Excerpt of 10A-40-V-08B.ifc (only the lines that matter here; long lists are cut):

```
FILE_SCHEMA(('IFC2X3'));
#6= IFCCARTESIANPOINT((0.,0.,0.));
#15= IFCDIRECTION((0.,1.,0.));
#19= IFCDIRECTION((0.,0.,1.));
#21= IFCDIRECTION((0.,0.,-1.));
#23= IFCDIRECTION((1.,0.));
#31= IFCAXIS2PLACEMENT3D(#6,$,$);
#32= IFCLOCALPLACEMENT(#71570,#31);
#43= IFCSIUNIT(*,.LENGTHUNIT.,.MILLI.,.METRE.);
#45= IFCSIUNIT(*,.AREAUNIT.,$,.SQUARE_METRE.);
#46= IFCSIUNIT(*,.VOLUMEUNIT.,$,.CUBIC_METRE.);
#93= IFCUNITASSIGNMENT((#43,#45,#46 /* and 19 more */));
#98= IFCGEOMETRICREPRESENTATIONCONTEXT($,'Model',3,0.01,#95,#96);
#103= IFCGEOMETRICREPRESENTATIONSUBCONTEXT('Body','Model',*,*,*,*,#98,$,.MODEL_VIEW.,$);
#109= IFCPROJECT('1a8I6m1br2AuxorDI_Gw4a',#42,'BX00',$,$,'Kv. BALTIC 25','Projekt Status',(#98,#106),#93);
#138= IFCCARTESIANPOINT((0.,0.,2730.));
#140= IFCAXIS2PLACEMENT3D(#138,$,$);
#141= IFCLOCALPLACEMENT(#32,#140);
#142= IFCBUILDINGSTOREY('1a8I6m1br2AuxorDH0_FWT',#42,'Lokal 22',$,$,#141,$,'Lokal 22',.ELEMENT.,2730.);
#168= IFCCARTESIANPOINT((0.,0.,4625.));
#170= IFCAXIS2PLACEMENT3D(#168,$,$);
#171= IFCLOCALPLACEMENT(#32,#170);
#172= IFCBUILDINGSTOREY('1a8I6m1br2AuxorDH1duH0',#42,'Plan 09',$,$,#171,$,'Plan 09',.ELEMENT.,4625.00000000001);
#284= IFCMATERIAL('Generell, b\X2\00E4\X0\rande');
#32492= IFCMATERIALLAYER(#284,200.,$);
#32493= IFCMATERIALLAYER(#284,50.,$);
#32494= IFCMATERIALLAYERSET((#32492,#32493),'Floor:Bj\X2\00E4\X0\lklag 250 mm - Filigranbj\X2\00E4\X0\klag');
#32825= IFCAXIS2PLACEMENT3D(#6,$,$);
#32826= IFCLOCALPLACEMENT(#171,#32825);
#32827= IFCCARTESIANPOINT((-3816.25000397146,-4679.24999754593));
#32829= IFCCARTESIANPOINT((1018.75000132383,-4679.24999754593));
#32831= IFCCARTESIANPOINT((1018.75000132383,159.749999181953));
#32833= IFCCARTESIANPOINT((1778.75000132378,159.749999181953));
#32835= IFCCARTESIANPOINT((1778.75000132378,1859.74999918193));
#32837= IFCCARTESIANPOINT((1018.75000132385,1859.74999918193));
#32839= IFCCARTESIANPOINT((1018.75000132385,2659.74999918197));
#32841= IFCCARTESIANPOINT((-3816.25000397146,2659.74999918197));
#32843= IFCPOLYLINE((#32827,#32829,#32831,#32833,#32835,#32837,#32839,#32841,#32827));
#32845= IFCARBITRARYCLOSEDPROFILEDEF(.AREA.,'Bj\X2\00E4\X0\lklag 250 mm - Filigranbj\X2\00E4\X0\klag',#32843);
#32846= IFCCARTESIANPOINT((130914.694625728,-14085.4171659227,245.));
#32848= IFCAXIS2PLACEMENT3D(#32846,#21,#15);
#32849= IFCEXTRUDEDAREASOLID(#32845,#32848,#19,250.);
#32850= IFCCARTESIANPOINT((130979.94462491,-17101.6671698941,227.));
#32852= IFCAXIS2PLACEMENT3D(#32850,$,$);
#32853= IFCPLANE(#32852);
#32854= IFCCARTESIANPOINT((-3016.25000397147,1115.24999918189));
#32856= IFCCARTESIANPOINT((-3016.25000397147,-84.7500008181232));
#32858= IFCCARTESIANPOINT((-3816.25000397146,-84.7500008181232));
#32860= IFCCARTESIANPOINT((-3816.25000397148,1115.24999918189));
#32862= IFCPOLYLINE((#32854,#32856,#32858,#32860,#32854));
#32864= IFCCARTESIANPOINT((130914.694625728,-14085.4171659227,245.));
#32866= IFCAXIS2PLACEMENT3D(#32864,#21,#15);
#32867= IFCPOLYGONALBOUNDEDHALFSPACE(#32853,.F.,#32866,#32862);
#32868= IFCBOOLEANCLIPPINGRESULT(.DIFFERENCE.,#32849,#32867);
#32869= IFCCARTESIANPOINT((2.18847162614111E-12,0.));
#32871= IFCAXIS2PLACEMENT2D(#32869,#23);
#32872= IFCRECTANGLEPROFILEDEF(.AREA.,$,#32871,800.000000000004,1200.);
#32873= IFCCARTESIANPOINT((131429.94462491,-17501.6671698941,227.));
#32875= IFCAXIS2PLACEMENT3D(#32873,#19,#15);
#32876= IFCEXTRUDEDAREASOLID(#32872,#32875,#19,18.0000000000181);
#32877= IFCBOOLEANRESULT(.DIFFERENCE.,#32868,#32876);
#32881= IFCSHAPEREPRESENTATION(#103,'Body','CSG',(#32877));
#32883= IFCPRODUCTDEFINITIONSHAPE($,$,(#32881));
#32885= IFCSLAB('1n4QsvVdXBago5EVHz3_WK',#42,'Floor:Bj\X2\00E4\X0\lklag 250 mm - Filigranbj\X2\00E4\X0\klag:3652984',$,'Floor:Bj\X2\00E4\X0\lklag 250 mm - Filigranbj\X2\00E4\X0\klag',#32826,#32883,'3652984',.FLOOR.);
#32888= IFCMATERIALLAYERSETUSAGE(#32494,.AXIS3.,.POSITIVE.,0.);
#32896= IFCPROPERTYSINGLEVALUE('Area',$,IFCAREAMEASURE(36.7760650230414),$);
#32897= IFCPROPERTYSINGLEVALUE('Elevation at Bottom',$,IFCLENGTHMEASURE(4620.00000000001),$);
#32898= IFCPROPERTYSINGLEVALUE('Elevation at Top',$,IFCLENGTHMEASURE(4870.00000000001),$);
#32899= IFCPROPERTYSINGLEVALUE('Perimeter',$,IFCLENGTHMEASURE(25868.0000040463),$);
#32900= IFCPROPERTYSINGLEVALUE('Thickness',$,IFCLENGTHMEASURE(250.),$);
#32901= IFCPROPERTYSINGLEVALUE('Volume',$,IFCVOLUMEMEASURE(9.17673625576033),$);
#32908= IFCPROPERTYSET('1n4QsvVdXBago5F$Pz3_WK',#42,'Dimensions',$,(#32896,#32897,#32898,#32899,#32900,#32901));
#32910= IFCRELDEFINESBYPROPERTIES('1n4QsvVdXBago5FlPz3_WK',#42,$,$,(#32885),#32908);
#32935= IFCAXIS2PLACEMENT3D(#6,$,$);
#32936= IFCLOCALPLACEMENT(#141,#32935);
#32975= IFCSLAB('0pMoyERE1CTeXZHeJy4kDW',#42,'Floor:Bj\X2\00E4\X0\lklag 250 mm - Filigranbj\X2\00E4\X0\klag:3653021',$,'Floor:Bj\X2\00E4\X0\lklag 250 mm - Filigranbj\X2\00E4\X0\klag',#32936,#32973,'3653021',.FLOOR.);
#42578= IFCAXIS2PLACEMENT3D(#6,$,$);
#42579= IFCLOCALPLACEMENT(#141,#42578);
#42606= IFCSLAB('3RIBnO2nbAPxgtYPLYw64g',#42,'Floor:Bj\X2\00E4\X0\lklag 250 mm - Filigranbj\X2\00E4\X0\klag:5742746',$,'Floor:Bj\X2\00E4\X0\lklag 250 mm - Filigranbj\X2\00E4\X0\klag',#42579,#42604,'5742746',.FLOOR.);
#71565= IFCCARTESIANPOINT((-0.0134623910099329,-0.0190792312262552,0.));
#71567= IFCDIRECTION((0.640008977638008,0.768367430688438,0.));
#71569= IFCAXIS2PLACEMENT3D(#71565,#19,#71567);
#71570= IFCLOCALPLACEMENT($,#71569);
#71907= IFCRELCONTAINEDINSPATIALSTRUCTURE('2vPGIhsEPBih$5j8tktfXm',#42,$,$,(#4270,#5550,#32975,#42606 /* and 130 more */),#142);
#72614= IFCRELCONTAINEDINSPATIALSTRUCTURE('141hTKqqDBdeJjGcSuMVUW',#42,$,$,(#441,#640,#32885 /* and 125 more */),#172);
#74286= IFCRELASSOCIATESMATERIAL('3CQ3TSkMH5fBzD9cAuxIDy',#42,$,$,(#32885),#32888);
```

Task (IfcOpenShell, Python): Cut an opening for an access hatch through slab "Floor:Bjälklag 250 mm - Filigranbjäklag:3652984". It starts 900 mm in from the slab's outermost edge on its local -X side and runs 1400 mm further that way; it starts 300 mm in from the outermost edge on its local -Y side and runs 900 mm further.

```python
import numpy as np
import ifcopenshell
import ifcopenshell.api.feature
import ifcopenshell.api.geometry
import ifcopenshell.api.pset
import ifcopenshell.api.root
import ifcopenshell.geom
import ifcopenshell.util.element
import ifcopenshell.util.placement
import ifcopenshell.util.representation
import ifcopenshell.util.shape
import ifcopenshell.util.unit

model = ifcopenshell.open("10A-40-V-08B.ifc")
unit_scale = ifcopenshell.util.unit.calculate_unit_scale(model)
area_scale = ifcopenshell.util.unit.calculate_unit_scale(model, "AREAUNIT")
volume_scale = ifcopenshell.util.unit.calculate_unit_scale(model, "VOLUMEUNIT")
settings = ifcopenshell.geom.settings()


def volume(element):
    """Net volume in cubic metres, openings subtracted."""
    shape = ifcopenshell.geom.create_shape(settings, element)
    return ifcopenshell.util.shape.get_volume(shape.geometry)


slab = model.by_guid("1n4QsvVdXBago5EVHz3_WK")
before = volume(slab)

# Extent in the slab's own axes, in metres. The edges named are its -X and -Y sides.
slab_shape = ifcopenshell.geom.create_shape(settings, slab)
vertices = ifcopenshell.util.shape.get_vertices(slab_shape.geometry)
x_min, y_min, bottom = vertices.min(axis=0)
top = vertices[:, 2].max()

opening = ifcopenshell.api.root.create_entity(model, ifc_class="IfcOpeningElement", name="Access hatch opening")
context = ifcopenshell.util.representation.get_context(model, "Model", "Body", "MODEL_VIEW")
width, depth = 1.4, 0.9
outline = [(0.0, 0.0), (width, 0.0), (width, depth), (0.0, depth), (0.0, 0.0)]
# Overshoot both faces by 50 mm so the cut is clean.
shape = ifcopenshell.api.geometry.add_slab_representation(
    model, context=context, depth=top - bottom + 0.1, polyline=outline
)
ifcopenshell.api.geometry.assign_representation(model, product=opening, representation=shape)

matrix = ifcopenshell.util.placement.get_local_placement(slab.ObjectPlacement)
matrix[:, 3] = matrix @ np.append(np.array([x_min + 0.9, y_min + 0.3, bottom - 0.05]) / unit_scale, 1.0)
ifcopenshell.api.geometry.edit_object_placement(model, product=opening, matrix=matrix, is_si=False)
ifcopenshell.api.feature.add_feature(model, feature=opening, element=slab)

after = volume(slab)

# Update the slab's stored quantities.
pset = model.by_id(ifcopenshell.util.element.get_pset(slab, "Dimensions", should_inherit=False)["id"])
ifcopenshell.api.pset.edit_pset(model, pset=pset, properties={
    "Area": model.create_entity("IfcAreaMeasure", after / (top - bottom) / area_scale),
    "Volume": model.create_entity("IfcVolumeMeasure", after / volume_scale),
})

print(f"slab volume {before:.3f} -> {after:.3f} m3")

model.write("10A-40-V-08B_edited.ifc")
```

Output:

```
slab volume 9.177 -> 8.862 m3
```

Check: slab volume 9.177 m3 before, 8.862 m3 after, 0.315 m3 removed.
